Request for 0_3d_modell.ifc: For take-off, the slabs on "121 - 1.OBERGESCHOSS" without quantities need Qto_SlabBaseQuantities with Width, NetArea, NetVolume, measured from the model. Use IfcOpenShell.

First a look at what the model holds.

```python
import ifcopenshell
import ifcopenshell.util.element
import ifcopenshell.util.unit

model = ifcopenshell.open("0_3d_modell.ifc")
print(model.schema)
for unit_type in ("LENGTHUNIT", "AREAUNIT", "VOLUMEUNIT"):
    print(unit_type, ifcopenshell.util.unit.calculate_unit_scale(model, unit_type))
storey = next(s for s in model.by_type("IfcBuildingStorey") if s.Name == "121 - 1.OBERGESCHOSS")
slabs = [e for e in ifcopenshell.util.element.get_decomposition(storey) if e.is_a("IfcSlab")]
for e in sorted(slabs, key=lambda e: e.id()):
    print(e.id(), e.is_a(), e.Name, list(ifcopenshell.util.element.get_psets(e, qtos_only=True)), sep=" | ")
```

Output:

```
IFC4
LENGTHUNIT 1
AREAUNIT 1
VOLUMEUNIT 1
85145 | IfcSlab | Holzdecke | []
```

```python
import ifcopenshell
import ifcopenshell.api.pset
import ifcopenshell.geom
import ifcopenshell.util.element
import ifcopenshell.util.shape
import ifcopenshell.util.unit

model = ifcopenshell.open("0_3d_modell.ifc")
unit_scale = ifcopenshell.util.unit.calculate_unit_scale(model)
area_scale = ifcopenshell.util.unit.calculate_unit_scale(model, "AREAUNIT")
volume_scale = ifcopenshell.util.unit.calculate_unit_scale(model, "VOLUMEUNIT")
settings = ifcopenshell.geom.settings()

storey = next(s for s in model.by_type("IfcBuildingStorey") if s.Name == "121 - 1.OBERGESCHOSS")
slabs = [e for e in ifcopenshell.util.element.get_decomposition(storey) if e.is_a("IfcSlab")]

for e in sorted(slabs, key=lambda e: e.id()):
    if ifcopenshell.util.element.get_psets(e, qtos_only=True, should_inherit=False):
        continue
    # Geometry comes back in metres, in the element's own axes.
    shape = ifcopenshell.geom.create_shape(settings, e)
    values = {
        "Width": ifcopenshell.util.shape.get_z(shape.geometry) / unit_scale,
        "NetArea": ifcopenshell.util.shape.get_footprint_area(shape.geometry) / area_scale,
        "NetVolume": ifcopenshell.util.shape.get_volume(shape.geometry) / volume_scale,
    }
    qto = ifcopenshell.api.pset.add_qto(model, product=e, name="Qto_SlabBaseQuantities")
    ifcopenshell.api.pset.edit_qto(model, qto=qto, properties=values)
    print(e.id(), {k: round(v, 3) for k, v in values.items()})

model.write("0_3d_modell_updated.ifc")
```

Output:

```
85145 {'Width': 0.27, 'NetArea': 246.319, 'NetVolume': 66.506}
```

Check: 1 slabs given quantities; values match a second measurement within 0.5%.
